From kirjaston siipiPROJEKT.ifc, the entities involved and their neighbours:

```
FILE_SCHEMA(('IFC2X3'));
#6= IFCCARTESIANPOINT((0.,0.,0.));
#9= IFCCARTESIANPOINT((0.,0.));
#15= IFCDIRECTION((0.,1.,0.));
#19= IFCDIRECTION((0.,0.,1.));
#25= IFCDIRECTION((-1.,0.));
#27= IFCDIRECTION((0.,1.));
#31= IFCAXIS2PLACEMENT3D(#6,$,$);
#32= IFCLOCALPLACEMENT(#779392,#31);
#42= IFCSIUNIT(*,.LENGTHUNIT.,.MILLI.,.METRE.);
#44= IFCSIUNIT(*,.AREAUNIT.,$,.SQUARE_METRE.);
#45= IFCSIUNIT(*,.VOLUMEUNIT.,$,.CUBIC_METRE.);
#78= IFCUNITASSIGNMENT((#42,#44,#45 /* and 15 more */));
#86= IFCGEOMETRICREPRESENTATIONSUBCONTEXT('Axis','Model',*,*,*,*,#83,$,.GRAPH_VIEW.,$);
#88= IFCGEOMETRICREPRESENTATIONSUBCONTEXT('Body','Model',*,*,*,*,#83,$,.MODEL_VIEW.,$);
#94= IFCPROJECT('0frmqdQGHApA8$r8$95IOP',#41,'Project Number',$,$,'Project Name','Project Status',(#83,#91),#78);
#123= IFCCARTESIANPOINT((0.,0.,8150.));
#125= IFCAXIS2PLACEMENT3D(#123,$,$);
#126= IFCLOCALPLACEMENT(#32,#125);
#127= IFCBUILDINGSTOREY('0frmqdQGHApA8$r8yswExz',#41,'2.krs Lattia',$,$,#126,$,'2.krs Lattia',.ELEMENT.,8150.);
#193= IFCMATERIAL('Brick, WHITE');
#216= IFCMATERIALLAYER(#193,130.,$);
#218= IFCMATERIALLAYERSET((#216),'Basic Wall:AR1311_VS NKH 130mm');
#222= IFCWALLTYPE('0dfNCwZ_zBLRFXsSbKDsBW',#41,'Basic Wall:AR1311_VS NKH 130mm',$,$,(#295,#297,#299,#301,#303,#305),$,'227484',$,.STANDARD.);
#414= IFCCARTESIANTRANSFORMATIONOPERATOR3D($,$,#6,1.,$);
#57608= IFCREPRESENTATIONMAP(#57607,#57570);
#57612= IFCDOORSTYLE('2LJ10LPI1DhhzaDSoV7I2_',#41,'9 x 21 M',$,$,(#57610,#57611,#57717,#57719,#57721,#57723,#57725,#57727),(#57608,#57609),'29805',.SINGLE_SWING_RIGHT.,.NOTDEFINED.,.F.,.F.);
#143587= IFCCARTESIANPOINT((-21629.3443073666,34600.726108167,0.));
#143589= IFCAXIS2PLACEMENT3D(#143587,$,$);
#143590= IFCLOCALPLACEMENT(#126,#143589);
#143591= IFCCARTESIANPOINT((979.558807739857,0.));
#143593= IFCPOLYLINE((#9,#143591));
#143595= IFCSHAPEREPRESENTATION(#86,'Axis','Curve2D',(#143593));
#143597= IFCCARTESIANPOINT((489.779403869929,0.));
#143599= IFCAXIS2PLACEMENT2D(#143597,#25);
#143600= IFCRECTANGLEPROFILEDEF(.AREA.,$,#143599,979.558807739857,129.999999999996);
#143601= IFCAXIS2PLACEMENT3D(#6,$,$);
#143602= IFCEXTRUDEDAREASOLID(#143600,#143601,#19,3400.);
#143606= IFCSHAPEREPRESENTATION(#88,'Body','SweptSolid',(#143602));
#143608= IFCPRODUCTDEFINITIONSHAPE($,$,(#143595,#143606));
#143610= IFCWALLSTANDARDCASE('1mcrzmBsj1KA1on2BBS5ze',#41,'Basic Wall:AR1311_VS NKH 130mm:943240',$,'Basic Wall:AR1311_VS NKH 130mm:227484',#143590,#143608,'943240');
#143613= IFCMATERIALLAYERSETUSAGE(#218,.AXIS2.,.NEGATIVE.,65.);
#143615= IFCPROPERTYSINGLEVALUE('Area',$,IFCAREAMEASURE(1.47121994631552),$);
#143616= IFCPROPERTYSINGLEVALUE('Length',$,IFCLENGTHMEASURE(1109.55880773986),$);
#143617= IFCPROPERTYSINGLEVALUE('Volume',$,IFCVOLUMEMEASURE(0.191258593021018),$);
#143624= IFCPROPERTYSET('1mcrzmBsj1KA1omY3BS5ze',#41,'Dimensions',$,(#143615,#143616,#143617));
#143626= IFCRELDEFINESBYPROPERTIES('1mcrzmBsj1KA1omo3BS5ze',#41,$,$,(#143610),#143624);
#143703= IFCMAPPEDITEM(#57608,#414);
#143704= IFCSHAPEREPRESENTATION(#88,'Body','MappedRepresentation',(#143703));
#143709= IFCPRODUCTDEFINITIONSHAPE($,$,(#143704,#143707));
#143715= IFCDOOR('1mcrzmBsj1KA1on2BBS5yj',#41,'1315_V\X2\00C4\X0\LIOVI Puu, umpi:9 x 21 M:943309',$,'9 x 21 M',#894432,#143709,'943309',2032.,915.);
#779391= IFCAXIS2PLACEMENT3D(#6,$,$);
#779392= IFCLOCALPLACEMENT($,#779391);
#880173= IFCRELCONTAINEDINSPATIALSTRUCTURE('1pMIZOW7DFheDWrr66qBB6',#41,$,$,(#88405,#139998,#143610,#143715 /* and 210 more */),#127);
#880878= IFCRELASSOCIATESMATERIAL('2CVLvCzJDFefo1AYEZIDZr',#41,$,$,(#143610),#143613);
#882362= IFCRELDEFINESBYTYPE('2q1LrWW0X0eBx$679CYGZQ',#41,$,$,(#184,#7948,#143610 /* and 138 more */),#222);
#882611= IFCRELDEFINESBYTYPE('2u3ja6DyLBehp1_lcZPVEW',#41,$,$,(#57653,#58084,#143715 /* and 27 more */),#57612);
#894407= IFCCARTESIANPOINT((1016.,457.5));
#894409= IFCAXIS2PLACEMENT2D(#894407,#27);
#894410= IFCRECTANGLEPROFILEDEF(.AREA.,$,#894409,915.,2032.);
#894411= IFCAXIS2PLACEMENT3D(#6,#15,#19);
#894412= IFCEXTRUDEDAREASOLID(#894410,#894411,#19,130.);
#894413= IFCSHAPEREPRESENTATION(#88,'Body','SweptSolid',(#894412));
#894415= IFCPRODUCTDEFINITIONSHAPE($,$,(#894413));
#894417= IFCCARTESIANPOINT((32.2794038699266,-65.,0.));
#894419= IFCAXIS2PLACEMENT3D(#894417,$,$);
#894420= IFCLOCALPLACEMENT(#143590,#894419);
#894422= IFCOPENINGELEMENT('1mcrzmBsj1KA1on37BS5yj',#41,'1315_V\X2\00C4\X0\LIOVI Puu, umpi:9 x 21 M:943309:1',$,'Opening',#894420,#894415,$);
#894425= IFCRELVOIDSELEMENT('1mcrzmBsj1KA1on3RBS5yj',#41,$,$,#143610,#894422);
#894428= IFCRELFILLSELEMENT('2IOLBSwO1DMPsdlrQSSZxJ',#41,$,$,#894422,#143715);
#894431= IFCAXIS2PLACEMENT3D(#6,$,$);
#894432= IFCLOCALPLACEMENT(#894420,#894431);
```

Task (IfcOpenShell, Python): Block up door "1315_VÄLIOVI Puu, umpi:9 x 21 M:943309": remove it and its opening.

```python
import ifcopenshell
import ifcopenshell.api.feature
import ifcopenshell.api.pset
import ifcopenshell.api.root
import ifcopenshell.geom
import ifcopenshell.util.element
import ifcopenshell.util.shape
import ifcopenshell.util.unit

model = ifcopenshell.open("kirjaston siipiPROJEKT.ifc")
area_scale = ifcopenshell.util.unit.calculate_unit_scale(model, "AREAUNIT")
volume_scale = ifcopenshell.util.unit.calculate_unit_scale(model, "VOLUMEUNIT")
settings = ifcopenshell.geom.settings()


def volume(element):
    """Net volume in cubic metres, openings subtracted."""
    shape = ifcopenshell.geom.create_shape(settings, element)
    return ifcopenshell.util.shape.get_volume(shape.geometry)


door = model.by_guid("1mcrzmBsj1KA1on2BBS5yj")
opening = door.FillsVoids[0].RelatingOpeningElement
wall = opening.VoidsElements[0].RelatingBuildingElement
before = volume(wall)

ifcopenshell.api.root.remove_product(model, product=door)
ifcopenshell.api.feature.remove_feature(model, feature=opening)

after = volume(wall)
thickness = 0.13  # wall thickness in metres

# Update the wall's stored quantities.
pset = model.by_id(ifcopenshell.util.element.get_pset(wall, "Dimensions", should_inherit=False)["id"])
ifcopenshell.api.pset.edit_pset(model, pset=pset, properties={
    "Area": model.create_entity("IfcAreaMeasure", after / thickness / area_scale),
    "Volume": model.create_entity("IfcVolumeMeasure", after / volume_scale),
})

print(f"wall volume {before:.3f} -> {after:.3f} m3")

model.write("kirjaston siipiPROJEKT-out.ifc")
```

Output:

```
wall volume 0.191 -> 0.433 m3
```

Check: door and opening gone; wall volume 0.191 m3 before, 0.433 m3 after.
